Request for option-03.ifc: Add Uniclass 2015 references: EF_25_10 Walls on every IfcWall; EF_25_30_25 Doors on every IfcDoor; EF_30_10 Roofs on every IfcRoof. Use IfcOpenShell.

First a look at what the model holds.

```python
import ifcopenshell

model = ifcopenshell.open("option-03.ifc")
print(model.schema)
print("classifications:", [c.Name for c in model.by_type("IfcClassification")])
for ifc_class in ("IfcDoor", "IfcRoof", "IfcStair", "IfcWall", "IfcWindow"):
    print(ifc_class, len(model.by_type(ifc_class)))
```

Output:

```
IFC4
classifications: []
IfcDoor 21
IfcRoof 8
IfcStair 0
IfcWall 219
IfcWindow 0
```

```python
import ifcopenshell
import ifcopenshell.api.classification

model = ifcopenshell.open("option-03.ifc")

system = ifcopenshell.api.classification.add_classification(model, classification="Uniclass 2015")

codes = {
    "IfcWall": ("EF_25_10", "Walls"),
    "IfcDoor": ("EF_25_30_25", "Doors"),
    "IfcRoof": ("EF_30_10", "Roofs"),
}
for ifc_class, (code, name) in codes.items():
    products = model.by_type(ifc_class)
    ifcopenshell.api.classification.add_reference(
        model, products=products, classification=system, identification=code, name=name
    )
    print(code, len(products))

model.write("option-03_updated.ifc")
```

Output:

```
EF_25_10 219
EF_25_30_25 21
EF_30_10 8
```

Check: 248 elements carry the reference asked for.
